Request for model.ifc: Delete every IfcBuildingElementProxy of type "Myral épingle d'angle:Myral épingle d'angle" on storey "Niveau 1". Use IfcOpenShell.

First a look at what the model holds.

```python
import ifcopenshell
import ifcopenshell.util.element

model = ifcopenshell.open("model.ifc")
print(model.schema)
storey = next(s for s in model.by_type("IfcBuildingStorey") if s.Name == "Niveau 1")
proxies = [e for e in ifcopenshell.util.element.get_decomposition(storey) if e.is_a("IfcBuildingElementProxy")]
seen = {}
for e in proxies:
    element_type = ifcopenshell.util.element.get_type(e)
    name = element_type.Name if element_type not in (None, e) else None
    seen[name] = seen.get(name, 0) + 1
for name, count in sorted(seen.items(), key=str):
    print(count, "x", name)
```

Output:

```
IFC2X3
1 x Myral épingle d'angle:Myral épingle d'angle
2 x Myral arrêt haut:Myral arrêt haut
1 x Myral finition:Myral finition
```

```python
import ifcopenshell
import ifcopenshell.api.root
import ifcopenshell.util.element

model = ifcopenshell.open("model.ifc")

storey = next(s for s in model.by_type("IfcBuildingStorey") if s.Name == "Niveau 1")
proxies = [e for e in ifcopenshell.util.element.get_decomposition(storey) if e.is_a("IfcBuildingElementProxy")]
targets = [e for e in proxies if (t := ifcopenshell.util.element.get_type(e)) not in (None, e) and t.Name == "Myral épingle d'angle:Myral épingle d'angle"]

for e in targets:
    ifcopenshell.api.root.remove_product(model, product=e)
print(len(targets), "removed")

model.write("model-out.ifc")
```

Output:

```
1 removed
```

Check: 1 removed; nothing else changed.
